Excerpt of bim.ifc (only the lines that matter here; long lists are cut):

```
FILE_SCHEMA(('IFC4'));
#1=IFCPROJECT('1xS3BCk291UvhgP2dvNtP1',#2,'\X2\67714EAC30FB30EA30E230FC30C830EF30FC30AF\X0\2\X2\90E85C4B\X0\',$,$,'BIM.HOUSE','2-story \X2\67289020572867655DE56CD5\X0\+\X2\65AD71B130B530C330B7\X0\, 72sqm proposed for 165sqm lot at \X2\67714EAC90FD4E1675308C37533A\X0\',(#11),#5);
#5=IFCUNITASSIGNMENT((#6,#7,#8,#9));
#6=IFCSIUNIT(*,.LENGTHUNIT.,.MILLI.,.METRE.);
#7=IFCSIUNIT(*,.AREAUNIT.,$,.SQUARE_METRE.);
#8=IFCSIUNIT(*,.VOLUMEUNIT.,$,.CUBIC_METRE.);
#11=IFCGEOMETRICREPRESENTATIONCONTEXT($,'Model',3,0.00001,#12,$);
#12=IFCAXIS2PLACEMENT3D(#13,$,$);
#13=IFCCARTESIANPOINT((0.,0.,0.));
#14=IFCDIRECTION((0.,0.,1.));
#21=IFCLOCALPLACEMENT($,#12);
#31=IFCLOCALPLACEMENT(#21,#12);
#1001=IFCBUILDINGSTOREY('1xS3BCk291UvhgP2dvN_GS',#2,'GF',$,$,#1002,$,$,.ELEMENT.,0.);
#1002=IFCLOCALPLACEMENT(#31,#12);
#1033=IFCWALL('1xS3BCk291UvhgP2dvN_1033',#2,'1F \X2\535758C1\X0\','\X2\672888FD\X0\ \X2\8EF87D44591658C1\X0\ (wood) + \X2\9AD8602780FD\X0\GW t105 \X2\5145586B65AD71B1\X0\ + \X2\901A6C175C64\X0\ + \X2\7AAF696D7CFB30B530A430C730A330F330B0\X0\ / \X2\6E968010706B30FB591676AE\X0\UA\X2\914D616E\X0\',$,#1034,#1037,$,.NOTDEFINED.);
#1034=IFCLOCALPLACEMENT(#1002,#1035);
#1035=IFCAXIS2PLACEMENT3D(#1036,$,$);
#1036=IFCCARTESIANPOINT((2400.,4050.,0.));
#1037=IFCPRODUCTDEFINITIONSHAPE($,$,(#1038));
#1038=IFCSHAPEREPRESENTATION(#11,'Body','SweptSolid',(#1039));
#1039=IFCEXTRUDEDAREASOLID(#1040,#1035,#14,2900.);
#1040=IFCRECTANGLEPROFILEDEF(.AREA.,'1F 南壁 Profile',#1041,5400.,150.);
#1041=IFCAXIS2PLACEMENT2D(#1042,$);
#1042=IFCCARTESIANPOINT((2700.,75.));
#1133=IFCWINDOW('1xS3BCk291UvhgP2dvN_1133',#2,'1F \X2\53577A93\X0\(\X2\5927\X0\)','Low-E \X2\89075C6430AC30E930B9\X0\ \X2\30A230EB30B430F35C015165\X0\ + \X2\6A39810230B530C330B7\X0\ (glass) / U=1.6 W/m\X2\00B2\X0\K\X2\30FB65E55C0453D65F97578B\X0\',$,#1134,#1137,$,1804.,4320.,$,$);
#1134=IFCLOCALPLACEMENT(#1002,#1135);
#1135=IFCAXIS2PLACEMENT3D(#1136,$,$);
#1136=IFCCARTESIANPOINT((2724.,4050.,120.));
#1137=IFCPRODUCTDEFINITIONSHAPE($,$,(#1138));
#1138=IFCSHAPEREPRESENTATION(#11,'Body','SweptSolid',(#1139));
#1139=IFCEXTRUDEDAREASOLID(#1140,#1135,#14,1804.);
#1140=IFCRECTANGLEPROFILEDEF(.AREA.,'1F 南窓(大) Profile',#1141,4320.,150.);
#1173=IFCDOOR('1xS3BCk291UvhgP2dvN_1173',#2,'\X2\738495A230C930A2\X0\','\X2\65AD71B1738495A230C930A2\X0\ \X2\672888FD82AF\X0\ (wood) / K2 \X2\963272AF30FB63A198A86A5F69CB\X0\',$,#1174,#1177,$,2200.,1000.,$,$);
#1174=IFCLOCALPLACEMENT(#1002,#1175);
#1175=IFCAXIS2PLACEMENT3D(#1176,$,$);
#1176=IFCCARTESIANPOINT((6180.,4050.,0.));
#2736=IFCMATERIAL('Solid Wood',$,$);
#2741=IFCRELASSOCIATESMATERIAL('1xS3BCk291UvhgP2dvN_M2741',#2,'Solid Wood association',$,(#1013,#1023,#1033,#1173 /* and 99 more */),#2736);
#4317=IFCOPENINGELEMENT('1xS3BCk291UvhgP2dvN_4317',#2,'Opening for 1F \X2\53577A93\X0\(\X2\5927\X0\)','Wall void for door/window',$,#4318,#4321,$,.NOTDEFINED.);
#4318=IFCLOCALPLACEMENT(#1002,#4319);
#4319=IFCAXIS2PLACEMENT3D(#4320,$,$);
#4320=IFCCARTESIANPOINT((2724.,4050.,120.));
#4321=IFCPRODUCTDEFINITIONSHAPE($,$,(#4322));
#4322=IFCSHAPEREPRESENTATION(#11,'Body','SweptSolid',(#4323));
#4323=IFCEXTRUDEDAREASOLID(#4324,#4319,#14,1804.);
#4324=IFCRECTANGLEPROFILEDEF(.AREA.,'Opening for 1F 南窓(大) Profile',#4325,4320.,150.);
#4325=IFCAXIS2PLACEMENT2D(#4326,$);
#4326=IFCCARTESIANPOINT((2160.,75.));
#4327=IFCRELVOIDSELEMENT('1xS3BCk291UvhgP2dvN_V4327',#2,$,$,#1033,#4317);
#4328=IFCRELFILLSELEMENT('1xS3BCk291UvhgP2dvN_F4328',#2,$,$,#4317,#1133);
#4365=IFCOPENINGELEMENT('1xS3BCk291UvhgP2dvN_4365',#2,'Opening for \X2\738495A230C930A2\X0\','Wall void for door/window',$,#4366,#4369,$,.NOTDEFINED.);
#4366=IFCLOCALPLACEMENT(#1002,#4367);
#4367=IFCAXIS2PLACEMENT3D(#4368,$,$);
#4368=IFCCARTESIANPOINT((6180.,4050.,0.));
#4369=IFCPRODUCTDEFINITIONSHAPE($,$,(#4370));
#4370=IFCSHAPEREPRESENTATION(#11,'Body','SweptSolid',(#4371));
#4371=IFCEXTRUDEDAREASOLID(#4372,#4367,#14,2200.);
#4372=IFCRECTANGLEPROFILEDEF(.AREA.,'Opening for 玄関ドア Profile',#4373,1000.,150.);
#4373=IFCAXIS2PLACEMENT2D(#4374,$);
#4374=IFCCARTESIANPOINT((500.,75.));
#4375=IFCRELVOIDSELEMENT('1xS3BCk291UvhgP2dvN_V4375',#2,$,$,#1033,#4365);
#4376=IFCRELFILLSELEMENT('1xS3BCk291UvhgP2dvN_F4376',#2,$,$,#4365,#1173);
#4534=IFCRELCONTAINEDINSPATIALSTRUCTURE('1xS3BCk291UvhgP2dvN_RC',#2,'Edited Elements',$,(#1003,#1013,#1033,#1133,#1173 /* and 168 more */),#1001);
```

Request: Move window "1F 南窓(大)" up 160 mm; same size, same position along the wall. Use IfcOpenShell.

```python
import numpy as np
import ifcopenshell
import ifcopenshell.api.geometry
import ifcopenshell.util.placement
import ifcopenshell.util.unit

model = ifcopenshell.open("bim.ifc")
unit_scale = ifcopenshell.util.unit.calculate_unit_scale(model)

window = model.by_id(1133)
opening = window.FillsVoids[0].RelatingOpeningElement
dz = 0.16 / unit_scale

shift = np.array([0.0, 0.0, dz])
# The window is not placed relative to its opening, so move both.
for product in (opening, window):
    matrix = ifcopenshell.util.placement.get_local_placement(product.ObjectPlacement)
    matrix[:3, 3] += shift
    ifcopenshell.api.geometry.edit_object_placement(model, product=product, matrix=matrix, is_si=False)

print(f"moved by {dz * unit_scale:+.3f} m")

model.write("bim_updated.ifc")
```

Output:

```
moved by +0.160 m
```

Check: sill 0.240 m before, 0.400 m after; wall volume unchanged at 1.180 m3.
